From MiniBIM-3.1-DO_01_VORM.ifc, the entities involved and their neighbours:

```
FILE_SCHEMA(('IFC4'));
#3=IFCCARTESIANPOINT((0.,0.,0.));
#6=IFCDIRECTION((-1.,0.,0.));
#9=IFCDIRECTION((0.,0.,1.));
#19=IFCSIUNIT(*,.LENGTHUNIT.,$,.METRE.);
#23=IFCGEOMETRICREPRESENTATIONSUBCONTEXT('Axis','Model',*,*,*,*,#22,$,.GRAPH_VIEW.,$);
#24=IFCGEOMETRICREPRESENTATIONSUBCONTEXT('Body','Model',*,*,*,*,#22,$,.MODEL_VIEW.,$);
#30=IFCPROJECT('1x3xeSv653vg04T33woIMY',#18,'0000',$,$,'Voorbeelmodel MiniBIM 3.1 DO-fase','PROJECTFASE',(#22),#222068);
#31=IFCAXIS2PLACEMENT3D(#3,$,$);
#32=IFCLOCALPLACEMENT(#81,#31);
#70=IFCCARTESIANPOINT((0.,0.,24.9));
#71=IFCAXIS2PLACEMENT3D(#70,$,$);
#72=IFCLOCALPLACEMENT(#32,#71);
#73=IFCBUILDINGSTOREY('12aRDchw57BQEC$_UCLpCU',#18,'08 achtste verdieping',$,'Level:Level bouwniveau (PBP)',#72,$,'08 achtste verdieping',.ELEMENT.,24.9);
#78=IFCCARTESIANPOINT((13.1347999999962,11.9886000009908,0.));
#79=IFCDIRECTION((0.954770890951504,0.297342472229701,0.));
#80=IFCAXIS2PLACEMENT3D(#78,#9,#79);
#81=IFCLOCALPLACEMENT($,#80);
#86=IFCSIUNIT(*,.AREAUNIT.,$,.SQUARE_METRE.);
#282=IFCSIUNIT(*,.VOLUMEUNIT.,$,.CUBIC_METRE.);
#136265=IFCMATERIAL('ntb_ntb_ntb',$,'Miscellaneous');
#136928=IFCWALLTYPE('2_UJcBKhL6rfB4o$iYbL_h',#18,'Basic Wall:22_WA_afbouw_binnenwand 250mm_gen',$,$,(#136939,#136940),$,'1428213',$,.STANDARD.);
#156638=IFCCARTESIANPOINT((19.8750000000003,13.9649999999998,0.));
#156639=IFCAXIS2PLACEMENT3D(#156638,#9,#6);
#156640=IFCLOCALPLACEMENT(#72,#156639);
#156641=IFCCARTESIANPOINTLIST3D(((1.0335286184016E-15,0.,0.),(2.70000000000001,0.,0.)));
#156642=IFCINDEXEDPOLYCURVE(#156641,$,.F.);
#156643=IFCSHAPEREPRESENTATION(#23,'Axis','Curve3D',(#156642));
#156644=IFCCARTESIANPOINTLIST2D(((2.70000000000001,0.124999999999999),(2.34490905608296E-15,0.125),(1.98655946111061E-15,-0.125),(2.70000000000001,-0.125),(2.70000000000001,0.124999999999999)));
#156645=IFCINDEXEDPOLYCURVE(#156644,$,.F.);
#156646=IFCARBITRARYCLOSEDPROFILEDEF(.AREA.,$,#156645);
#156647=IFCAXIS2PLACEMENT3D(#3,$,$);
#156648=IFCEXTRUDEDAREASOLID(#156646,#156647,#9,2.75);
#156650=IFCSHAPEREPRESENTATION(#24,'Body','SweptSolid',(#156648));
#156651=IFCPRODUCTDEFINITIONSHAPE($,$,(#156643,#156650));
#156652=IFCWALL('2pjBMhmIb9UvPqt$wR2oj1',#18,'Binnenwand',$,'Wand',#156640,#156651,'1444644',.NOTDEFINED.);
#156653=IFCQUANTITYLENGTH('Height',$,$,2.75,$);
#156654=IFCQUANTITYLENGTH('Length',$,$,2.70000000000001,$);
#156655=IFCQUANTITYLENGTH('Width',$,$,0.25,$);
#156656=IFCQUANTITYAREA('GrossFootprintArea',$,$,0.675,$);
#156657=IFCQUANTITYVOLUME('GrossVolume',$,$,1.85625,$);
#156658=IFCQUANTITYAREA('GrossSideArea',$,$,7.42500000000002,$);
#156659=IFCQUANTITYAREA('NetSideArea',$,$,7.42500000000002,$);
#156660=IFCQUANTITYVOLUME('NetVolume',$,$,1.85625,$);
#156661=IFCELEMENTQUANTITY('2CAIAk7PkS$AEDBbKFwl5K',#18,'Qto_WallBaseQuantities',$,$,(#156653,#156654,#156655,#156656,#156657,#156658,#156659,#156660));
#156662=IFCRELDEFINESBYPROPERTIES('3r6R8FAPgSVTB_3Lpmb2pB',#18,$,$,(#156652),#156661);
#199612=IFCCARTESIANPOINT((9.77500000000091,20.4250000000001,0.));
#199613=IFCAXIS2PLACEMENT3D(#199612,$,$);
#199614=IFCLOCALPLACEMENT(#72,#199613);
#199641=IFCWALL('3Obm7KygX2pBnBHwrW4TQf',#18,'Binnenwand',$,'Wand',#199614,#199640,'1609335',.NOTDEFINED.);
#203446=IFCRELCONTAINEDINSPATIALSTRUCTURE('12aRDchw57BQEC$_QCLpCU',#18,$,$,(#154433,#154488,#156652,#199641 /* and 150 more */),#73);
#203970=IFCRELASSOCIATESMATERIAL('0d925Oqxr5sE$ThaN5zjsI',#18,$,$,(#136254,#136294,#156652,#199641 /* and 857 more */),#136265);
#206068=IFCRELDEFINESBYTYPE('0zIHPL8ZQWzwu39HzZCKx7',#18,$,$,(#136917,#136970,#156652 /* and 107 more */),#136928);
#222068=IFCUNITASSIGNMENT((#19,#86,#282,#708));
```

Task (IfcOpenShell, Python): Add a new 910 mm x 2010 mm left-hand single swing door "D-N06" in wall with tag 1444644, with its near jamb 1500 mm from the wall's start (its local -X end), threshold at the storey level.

```python
import numpy as np
import ifcopenshell
import ifcopenshell.api.feature
import ifcopenshell.api.geometry
import ifcopenshell.api.pset
import ifcopenshell.api.root
import ifcopenshell.api.spatial
import ifcopenshell.geom
import ifcopenshell.util.element
import ifcopenshell.util.placement
import ifcopenshell.util.representation
import ifcopenshell.util.shape
import ifcopenshell.util.unit

model = ifcopenshell.open("MiniBIM-3.1-DO_01_VORM.ifc")
unit_scale = ifcopenshell.util.unit.calculate_unit_scale(model)
area_scale = ifcopenshell.util.unit.calculate_unit_scale(model, "AREAUNIT")
volume_scale = ifcopenshell.util.unit.calculate_unit_scale(model, "VOLUMEUNIT")
settings = ifcopenshell.geom.settings()


def volume(element):
    """Net volume in cubic metres, openings subtracted."""
    shape = ifcopenshell.geom.create_shape(settings, element)
    return ifcopenshell.util.shape.get_volume(shape.geometry)


wall = model.by_guid("2pjBMhmIb9UvPqt$wR2oj1")
storey = ifcopenshell.util.element.get_container(wall, ifc_class="IfcBuildingStorey")
context = ifcopenshell.util.representation.get_context(model, "Model", "Body", "MODEL_VIEW")
before = volume(wall)

width, height, from_end, sill = 0.91, 2.01, 1.5, 0.0  # metres

# The wall runs along its own X axis, and the end named is its -X end.
wall_shape = ifcopenshell.geom.create_shape(settings, wall)
x, y, z = ifcopenshell.util.shape.get_vertices(wall_shape.geometry).T
start = x.min() + from_end
face, thickness = float(y.min()), float(y.max() - y.min())
wall_matrix = ifcopenshell.util.placement.get_local_placement(wall.ObjectPlacement)
level = ifcopenshell.util.placement.get_local_placement(storey.ObjectPlacement)[2, 3]


def in_wall(x, y):
    """Placement at x, y metres in the wall's axes, at sill height."""
    matrix = wall_matrix.copy()
    matrix[:, 3] = wall_matrix @ np.array([x / unit_scale, y / unit_scale, 0.0, 1.0])
    matrix[2, 3] = level + sill / unit_scale
    return matrix


# Opening: a box that overshoots both wall faces by 50 mm.
opening = ifcopenshell.api.root.create_entity(model, ifc_class="IfcOpeningElement", predefined_type="OPENING")
box = ifcopenshell.api.geometry.add_wall_representation(
    model, context=context, length=width, height=height, thickness=thickness + 0.1
)
ifcopenshell.api.geometry.assign_representation(model, product=opening, representation=box)
ifcopenshell.api.geometry.edit_object_placement(model, product=opening, matrix=in_wall(start, face - 0.05), is_si=False)
ifcopenshell.api.feature.add_feature(model, feature=opening, element=wall)

door = ifcopenshell.api.root.create_entity(model, ifc_class="IfcDoor", name="D-N06", predefined_type="DOOR")
door.OverallWidth, door.OverallHeight = width / unit_scale, height / unit_scale
door.OperationType = "SINGLE_SWING_LEFT"
body = ifcopenshell.api.geometry.add_door_representation(
    model,
    context=context,
    overall_width=door.OverallWidth,
    overall_height=door.OverallHeight,
    operation_type="SINGLE_SWING_LEFT",
    lining_properties={"LiningDepth": thickness / unit_scale, "ThresholdDepth": thickness / unit_scale},
)
ifcopenshell.api.geometry.assign_representation(model, product=door, representation=body)
ifcopenshell.api.spatial.assign_container(model, products=[door], relating_structure=storey)
ifcopenshell.api.feature.add_filling(model, opening=opening, element=door)

# The lining spans the wall, so the door starts at the wall face.
ifcopenshell.api.geometry.edit_object_placement(model, product=door, matrix=in_wall(start, face), is_si=False)

after = volume(wall)

# Update the wall's stored quantities.
qto = model.by_id(ifcopenshell.util.element.get_pset(wall, "Qto_WallBaseQuantities", should_inherit=False)["id"])
ifcopenshell.api.pset.edit_qto(model, qto=qto, properties={
    "NetSideArea": after / thickness / area_scale,
    "NetVolume": after / volume_scale,
})

print(f"wall volume {before:.3f} -> {after:.3f} m3")

model.write("MiniBIM-3.1-DO_01_VORM_updated.ifc")
```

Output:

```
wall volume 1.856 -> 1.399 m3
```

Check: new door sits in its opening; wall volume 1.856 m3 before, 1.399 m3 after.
